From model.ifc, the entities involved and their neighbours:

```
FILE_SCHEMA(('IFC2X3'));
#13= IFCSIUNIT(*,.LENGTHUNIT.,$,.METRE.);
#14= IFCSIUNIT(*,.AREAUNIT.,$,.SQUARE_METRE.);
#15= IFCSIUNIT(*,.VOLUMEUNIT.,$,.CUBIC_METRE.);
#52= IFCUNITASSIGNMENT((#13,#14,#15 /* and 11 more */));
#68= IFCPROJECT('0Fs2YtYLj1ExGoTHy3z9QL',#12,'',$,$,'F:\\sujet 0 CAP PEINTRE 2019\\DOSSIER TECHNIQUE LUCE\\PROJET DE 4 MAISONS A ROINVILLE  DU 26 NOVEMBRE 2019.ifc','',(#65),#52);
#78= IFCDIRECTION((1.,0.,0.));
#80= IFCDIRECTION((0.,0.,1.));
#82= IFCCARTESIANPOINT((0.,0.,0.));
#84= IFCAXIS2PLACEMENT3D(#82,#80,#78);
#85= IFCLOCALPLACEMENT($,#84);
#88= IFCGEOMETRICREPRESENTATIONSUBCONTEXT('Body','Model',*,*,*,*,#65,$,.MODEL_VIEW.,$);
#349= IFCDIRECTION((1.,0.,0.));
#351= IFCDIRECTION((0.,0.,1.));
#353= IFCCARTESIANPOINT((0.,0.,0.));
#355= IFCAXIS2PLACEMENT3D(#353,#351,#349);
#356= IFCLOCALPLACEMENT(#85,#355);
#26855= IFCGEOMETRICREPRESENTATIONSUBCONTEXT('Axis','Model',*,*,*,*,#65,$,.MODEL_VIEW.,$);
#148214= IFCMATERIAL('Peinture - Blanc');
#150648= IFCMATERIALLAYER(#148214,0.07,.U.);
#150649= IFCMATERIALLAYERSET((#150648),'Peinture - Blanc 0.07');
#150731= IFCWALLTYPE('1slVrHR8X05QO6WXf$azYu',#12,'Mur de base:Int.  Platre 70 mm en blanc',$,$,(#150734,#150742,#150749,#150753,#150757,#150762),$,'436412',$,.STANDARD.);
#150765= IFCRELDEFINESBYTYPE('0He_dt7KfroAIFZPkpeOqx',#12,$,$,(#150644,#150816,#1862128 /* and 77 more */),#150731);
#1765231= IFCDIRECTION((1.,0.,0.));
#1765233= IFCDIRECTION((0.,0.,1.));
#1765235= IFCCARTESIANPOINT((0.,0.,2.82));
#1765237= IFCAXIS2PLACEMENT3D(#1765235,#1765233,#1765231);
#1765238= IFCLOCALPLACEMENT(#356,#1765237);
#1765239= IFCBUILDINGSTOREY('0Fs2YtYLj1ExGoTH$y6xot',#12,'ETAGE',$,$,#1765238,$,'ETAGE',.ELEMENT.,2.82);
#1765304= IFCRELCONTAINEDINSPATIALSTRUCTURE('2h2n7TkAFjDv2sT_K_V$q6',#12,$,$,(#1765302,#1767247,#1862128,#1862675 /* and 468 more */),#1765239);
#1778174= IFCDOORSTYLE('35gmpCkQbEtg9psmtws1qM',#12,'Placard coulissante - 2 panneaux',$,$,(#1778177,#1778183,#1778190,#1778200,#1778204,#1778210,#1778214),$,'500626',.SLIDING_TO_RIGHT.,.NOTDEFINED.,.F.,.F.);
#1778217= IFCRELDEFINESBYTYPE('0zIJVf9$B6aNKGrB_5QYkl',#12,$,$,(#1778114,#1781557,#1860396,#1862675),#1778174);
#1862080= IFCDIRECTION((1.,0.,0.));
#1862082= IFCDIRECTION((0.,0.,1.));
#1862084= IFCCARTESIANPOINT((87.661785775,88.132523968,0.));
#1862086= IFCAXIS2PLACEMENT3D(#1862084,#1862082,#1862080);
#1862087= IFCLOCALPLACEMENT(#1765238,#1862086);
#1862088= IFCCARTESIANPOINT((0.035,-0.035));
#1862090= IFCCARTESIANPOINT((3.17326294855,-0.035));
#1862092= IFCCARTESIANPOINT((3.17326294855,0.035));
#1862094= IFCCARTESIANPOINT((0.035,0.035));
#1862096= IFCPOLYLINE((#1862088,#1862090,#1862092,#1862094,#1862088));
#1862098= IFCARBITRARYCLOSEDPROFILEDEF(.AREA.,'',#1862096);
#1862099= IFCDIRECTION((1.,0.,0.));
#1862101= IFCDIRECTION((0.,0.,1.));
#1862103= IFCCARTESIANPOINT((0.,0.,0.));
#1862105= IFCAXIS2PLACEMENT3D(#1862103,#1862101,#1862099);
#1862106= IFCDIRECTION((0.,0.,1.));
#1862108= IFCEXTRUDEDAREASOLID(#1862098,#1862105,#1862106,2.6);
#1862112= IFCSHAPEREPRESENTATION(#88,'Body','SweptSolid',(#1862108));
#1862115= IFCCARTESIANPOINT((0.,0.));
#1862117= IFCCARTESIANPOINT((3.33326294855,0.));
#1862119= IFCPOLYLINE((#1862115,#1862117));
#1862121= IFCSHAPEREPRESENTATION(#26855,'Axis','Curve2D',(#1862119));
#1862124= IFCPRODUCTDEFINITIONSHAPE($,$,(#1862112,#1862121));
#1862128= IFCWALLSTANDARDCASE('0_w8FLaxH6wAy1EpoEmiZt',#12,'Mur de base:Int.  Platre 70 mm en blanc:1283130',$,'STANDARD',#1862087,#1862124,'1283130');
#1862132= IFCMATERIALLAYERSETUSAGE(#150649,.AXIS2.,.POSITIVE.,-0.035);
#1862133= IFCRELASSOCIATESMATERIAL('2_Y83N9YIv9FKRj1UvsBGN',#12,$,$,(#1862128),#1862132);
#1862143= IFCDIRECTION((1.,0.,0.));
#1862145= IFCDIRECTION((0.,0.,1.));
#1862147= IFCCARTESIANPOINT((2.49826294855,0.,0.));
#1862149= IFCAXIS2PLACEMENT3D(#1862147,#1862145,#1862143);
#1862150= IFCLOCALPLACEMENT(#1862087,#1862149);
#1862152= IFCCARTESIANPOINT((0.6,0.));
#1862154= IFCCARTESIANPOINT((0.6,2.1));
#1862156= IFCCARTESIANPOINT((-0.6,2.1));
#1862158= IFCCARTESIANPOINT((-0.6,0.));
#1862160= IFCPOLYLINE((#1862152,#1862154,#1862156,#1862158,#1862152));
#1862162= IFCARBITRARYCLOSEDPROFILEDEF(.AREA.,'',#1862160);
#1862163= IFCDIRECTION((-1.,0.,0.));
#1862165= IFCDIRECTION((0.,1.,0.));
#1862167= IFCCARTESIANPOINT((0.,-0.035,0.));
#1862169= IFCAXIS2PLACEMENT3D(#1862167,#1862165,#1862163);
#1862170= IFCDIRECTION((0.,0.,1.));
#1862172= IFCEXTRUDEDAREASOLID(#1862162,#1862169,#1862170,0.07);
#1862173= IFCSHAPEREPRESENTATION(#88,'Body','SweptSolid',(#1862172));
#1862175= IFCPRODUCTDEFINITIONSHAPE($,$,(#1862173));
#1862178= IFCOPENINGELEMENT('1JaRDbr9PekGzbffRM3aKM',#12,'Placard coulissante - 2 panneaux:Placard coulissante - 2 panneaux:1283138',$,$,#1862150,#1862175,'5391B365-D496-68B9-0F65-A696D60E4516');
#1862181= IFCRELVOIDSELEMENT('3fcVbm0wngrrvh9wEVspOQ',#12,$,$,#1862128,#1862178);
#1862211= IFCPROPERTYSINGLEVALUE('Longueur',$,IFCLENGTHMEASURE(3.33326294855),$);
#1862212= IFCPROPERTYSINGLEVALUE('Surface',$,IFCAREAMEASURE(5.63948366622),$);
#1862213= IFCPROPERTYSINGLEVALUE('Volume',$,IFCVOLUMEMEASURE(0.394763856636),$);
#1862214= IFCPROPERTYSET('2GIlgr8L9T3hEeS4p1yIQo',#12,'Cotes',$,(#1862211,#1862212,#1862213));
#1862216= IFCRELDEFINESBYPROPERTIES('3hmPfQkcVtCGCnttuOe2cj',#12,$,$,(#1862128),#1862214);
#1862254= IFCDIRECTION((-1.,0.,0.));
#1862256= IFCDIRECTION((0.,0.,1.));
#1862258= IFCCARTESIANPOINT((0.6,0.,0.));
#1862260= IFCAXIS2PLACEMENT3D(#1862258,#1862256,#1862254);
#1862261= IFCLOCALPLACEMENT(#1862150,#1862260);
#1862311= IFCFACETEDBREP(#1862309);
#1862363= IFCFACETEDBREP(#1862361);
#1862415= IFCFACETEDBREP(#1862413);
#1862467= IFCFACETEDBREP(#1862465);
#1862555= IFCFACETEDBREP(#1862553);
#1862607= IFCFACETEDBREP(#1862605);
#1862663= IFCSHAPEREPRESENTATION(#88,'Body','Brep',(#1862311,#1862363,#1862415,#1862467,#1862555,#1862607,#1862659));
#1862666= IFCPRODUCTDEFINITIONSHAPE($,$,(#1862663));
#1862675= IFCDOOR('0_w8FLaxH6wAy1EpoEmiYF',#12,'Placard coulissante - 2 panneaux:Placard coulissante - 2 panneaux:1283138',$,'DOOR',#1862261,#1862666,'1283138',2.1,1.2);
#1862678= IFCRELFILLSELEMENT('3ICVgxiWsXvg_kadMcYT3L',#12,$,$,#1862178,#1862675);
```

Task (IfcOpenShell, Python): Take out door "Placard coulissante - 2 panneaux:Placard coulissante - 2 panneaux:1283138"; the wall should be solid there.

```python
import ifcopenshell
import ifcopenshell.api.feature
import ifcopenshell.api.pset
import ifcopenshell.api.root
import ifcopenshell.geom
import ifcopenshell.util.element
import ifcopenshell.util.shape
import ifcopenshell.util.unit

model = ifcopenshell.open("model.ifc")
area_scale = ifcopenshell.util.unit.calculate_unit_scale(model, "AREAUNIT")
volume_scale = ifcopenshell.util.unit.calculate_unit_scale(model, "VOLUMEUNIT")
settings = ifcopenshell.geom.settings()


def volume(element):
    """Net volume in cubic metres, openings subtracted."""
    shape = ifcopenshell.geom.create_shape(settings, element)
    return ifcopenshell.util.shape.get_volume(shape.geometry)


door = model.by_guid("0_w8FLaxH6wAy1EpoEmiYF")
opening = door.FillsVoids[0].RelatingOpeningElement
wall = opening.VoidsElements[0].RelatingBuildingElement
before = volume(wall)

ifcopenshell.api.root.remove_product(model, product=door)
ifcopenshell.api.feature.remove_feature(model, feature=opening)

after = volume(wall)
thickness = 0.07  # wall thickness in metres

# Update the wall's stored quantities.
pset = model.by_id(ifcopenshell.util.element.get_pset(wall, "Cotes", should_inherit=False)["id"])
ifcopenshell.api.pset.edit_pset(model, pset=pset, properties={
    "Surface": model.create_entity("IfcAreaMeasure", after / thickness / area_scale),
    "Volume": model.create_entity("IfcVolumeMeasure", after / volume_scale),
})

print(f"wall volume {before:.3f} -> {after:.3f} m3")

model.write("model_v2.ifc")
```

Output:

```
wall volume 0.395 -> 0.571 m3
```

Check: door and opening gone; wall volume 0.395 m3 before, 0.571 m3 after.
